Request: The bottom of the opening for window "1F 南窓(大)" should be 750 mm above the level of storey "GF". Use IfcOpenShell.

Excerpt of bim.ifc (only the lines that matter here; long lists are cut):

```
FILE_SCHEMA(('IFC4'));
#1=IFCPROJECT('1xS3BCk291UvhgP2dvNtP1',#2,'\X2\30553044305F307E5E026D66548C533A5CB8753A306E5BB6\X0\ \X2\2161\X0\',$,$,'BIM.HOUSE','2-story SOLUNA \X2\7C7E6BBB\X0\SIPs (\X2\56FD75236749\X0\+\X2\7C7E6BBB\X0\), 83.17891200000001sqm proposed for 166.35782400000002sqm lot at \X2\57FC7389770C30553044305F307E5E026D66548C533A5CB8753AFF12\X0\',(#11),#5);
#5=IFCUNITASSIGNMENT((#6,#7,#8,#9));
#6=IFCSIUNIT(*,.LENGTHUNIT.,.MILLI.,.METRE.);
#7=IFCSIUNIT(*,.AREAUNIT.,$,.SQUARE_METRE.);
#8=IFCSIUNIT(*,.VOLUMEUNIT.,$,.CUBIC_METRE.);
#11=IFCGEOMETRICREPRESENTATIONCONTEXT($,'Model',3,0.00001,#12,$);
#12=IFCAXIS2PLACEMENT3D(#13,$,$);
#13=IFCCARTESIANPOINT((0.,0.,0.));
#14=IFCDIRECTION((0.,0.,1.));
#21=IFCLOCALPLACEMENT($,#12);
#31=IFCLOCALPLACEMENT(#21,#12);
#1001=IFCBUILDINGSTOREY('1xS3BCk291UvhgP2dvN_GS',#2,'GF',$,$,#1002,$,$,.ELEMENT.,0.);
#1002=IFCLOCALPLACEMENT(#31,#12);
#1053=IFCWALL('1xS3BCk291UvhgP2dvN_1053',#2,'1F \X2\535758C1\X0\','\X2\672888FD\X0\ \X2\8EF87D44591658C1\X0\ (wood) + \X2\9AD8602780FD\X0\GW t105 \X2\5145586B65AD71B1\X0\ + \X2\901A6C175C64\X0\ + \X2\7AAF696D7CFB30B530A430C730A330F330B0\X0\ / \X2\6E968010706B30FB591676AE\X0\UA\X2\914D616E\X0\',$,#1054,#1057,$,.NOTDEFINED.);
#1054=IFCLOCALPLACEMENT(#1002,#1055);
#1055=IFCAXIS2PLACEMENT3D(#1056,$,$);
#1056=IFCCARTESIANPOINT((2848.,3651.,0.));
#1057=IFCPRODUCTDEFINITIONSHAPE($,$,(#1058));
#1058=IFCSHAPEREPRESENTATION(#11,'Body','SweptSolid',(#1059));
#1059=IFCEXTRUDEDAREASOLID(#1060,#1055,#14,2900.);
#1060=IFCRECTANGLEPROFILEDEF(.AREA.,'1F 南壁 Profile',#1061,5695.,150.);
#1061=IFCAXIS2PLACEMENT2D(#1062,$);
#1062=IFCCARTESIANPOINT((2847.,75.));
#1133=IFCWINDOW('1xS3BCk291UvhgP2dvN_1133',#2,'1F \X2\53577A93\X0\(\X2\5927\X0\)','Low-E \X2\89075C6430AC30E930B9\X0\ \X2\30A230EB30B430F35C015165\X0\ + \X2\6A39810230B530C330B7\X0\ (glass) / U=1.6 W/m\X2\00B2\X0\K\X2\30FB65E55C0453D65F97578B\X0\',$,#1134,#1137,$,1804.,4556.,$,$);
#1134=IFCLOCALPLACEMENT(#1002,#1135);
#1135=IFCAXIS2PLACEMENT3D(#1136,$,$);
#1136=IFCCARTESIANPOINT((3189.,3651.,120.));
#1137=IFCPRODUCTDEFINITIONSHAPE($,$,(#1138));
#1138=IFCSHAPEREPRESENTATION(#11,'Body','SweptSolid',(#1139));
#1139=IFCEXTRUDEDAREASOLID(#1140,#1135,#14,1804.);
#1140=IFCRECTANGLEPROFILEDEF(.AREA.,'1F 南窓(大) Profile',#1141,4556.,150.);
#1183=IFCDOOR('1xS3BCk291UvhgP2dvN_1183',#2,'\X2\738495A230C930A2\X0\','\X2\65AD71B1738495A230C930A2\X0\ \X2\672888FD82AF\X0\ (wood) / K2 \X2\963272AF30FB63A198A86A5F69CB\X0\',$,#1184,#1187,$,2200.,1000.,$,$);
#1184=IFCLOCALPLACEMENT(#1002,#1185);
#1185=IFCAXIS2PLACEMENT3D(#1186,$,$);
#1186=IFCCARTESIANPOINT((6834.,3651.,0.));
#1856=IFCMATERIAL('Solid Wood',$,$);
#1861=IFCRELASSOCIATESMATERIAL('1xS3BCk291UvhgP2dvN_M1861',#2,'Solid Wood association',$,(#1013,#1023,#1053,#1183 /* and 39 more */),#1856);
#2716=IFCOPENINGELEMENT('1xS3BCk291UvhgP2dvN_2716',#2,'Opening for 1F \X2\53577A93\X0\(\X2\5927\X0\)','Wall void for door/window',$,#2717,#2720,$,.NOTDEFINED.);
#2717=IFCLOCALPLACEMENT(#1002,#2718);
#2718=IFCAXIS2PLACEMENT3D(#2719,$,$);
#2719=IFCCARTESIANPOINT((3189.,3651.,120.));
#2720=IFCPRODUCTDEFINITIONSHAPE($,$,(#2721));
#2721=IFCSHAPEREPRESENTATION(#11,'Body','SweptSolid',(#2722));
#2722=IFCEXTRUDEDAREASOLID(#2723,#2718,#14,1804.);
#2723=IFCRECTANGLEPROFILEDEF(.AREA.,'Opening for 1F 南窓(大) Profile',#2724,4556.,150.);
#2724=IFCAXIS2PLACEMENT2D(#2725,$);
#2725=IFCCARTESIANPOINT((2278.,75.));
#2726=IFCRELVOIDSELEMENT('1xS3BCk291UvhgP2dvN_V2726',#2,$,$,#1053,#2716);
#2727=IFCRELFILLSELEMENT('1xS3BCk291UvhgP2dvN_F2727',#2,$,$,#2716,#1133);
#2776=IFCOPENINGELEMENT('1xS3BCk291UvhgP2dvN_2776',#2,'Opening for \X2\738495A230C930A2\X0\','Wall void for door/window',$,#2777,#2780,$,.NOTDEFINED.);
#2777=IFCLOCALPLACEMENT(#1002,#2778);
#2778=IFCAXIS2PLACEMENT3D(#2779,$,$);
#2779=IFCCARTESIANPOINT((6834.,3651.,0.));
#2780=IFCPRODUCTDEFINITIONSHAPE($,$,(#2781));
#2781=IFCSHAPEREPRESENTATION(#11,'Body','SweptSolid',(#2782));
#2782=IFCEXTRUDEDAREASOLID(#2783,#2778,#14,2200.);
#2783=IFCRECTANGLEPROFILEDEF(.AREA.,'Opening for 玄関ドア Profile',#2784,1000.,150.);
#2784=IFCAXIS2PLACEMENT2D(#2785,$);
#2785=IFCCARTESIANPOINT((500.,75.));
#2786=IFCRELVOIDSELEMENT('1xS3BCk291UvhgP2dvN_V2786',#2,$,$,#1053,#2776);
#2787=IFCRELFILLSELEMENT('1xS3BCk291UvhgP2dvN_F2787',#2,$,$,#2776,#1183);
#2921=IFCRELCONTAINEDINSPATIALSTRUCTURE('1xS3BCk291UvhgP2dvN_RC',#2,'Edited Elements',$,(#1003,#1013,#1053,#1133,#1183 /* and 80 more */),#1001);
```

```python
import numpy as np
import ifcopenshell
import ifcopenshell.api.geometry
import ifcopenshell.geom
import ifcopenshell.util.element
import ifcopenshell.util.placement
import ifcopenshell.util.shape
import ifcopenshell.util.unit

model = ifcopenshell.open("bim.ifc")
unit_scale = ifcopenshell.util.unit.calculate_unit_scale(model)

window = model.by_guid("1xS3BCk291UvhgP2dvN_1133")
opening = window.FillsVoids[0].RelatingOpeningElement
storey = ifcopenshell.util.element.get_container(window, ifc_class="IfcBuildingStorey")
level = ifcopenshell.util.placement.get_local_placement(storey.ObjectPlacement)[2, 3]

# The opening's origin need not be at the sill, so measure its lowest point.
shape = ifcopenshell.geom.create_shape(ifcopenshell.geom.settings(), opening)
bottom = ifcopenshell.util.shape.get_shape_bottom_elevation(shape, shape.geometry) / unit_scale
dz = level + 0.75 / unit_scale - bottom

shift = np.array([0.0, 0.0, dz])
# The window is not placed relative to its opening, so move both.
for product in (opening, window):
    matrix = ifcopenshell.util.placement.get_local_placement(product.ObjectPlacement)
    matrix[:3, 3] += shift
    ifcopenshell.api.geometry.edit_object_placement(model, product=product, matrix=matrix, is_si=False)

print(f"moved by {dz * unit_scale:+.3f} m")

model.write("bim_v2.ifc")
```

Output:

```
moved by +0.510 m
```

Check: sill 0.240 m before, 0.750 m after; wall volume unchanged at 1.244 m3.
